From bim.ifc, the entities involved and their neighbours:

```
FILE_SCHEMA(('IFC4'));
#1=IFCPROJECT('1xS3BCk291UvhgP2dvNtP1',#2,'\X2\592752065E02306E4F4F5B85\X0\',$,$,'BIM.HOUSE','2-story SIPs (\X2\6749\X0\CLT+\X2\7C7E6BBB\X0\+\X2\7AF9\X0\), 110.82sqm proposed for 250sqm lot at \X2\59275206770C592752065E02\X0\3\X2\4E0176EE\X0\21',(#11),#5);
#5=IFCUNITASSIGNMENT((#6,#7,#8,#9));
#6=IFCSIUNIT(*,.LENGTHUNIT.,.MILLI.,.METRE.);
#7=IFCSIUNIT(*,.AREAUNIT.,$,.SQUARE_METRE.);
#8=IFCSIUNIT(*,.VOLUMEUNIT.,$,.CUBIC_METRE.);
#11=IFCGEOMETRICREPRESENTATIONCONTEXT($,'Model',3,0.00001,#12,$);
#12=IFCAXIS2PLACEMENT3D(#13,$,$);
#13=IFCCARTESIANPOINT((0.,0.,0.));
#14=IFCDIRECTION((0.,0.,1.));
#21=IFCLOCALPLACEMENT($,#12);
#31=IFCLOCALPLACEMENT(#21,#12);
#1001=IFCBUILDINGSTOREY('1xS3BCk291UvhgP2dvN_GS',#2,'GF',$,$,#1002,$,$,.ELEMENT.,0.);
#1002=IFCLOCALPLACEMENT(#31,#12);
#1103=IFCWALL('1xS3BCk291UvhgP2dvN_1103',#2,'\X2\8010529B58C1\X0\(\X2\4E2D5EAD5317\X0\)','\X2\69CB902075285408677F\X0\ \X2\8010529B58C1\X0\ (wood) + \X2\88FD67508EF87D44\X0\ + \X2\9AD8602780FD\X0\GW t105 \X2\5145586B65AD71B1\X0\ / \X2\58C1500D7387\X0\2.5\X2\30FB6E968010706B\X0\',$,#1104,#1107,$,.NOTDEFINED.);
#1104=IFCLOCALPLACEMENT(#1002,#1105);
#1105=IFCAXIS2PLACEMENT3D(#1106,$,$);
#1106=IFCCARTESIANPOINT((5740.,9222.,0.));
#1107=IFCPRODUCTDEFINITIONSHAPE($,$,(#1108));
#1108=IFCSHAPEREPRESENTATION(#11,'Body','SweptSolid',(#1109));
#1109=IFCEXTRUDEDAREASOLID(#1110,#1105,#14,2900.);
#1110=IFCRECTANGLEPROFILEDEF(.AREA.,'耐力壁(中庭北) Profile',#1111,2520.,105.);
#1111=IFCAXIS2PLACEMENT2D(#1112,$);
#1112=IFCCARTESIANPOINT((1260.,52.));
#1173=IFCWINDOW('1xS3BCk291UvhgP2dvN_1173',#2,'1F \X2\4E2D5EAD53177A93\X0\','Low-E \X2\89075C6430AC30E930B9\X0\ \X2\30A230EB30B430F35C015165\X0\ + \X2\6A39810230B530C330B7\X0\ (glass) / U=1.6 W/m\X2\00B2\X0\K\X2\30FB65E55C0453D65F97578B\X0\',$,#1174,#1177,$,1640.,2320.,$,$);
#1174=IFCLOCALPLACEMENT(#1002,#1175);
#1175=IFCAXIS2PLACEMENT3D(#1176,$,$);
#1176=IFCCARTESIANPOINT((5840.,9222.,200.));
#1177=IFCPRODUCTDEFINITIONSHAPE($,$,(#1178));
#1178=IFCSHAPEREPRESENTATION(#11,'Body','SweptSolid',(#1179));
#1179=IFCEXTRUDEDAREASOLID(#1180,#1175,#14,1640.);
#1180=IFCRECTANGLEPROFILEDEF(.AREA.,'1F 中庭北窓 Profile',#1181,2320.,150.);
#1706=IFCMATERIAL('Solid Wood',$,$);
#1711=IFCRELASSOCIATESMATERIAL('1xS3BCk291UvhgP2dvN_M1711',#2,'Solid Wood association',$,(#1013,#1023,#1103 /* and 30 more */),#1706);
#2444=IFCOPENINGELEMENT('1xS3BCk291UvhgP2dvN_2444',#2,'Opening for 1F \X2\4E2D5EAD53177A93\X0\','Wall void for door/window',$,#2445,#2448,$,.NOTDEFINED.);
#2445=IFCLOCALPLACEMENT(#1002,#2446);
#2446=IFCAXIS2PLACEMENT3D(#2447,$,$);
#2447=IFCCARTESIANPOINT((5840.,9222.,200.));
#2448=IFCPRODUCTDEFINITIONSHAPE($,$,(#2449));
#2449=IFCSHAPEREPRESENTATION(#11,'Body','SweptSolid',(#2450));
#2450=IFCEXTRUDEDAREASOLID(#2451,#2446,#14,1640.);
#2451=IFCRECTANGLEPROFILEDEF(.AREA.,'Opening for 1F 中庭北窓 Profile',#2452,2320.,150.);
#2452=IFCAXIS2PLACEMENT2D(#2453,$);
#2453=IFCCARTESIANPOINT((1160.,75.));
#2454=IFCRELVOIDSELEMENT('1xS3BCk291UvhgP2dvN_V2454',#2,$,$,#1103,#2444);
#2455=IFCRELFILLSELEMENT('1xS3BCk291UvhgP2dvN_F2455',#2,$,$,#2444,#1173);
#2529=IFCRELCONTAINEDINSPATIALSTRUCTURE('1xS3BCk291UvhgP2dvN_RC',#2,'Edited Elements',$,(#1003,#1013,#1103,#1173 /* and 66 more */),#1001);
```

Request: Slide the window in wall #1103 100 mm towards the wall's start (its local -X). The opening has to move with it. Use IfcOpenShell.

```python
import ifcopenshell
import ifcopenshell.api.geometry
import ifcopenshell.util.placement
import ifcopenshell.util.unit

model = ifcopenshell.open("bim.ifc")
unit_scale = ifcopenshell.util.unit.calculate_unit_scale(model)

window = model.by_id(1173)
opening = window.FillsVoids[0].RelatingOpeningElement
wall = opening.VoidsElements[0].RelatingBuildingElement

wall_matrix = ifcopenshell.util.placement.get_local_placement(wall.ObjectPlacement)
shift = wall_matrix[:3, 0] * -0.1 / unit_scale
before = ifcopenshell.util.placement.get_local_placement(window.ObjectPlacement)[:3, 3].copy()

# The window is not placed relative to its opening, so move both.
for product in (opening, window):
    matrix = ifcopenshell.util.placement.get_local_placement(product.ObjectPlacement)
    matrix[:3, 3] += shift
    ifcopenshell.api.geometry.edit_object_placement(model, product=product, matrix=matrix, is_si=False)

after = ifcopenshell.util.placement.get_local_placement(window.ObjectPlacement)[:3, 3]
print("window moved by", (after - before).round(3) + 0.0)

model.write("bim-out.ifc")
```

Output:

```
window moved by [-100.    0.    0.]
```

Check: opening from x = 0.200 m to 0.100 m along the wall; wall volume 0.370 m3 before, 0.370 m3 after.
